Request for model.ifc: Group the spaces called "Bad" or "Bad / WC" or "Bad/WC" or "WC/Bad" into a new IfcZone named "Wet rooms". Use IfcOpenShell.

First a look at what the model holds.

```python
import ifcopenshell

model = ifcopenshell.open("model.ifc")
print(model.schema)
seen = {}
for space in model.by_type("IfcSpace"):
    seen[space.LongName] = seen.get(space.LongName, 0) + 1
for name, count in sorted(seen.items(), key=str):
    print(count, "x", name)
print("zones:", [z.Name for z in model.by_type("IfcZone")][:20])
```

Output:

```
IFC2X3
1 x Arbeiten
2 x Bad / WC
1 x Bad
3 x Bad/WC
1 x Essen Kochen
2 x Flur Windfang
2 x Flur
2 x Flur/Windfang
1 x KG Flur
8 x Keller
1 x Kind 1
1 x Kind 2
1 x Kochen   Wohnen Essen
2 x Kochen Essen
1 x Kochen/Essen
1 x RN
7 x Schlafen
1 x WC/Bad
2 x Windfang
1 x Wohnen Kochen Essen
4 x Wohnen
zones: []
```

```python
import ifcopenshell
import ifcopenshell.api.group
import ifcopenshell.api.root

model = ifcopenshell.open("model.ifc")

names = {"Bad", "Bad / WC", "Bad/WC", "WC/Bad"}
spaces = [s for s in model.by_type("IfcSpace") if s.LongName in names]

zone = ifcopenshell.api.root.create_entity(model, ifc_class="IfcZone", name="Wet rooms")
ifcopenshell.api.group.assign_group(model, products=spaces, group=zone)
print(len(spaces), "spaces in", zone.Name)

model.write("model_v2.ifc")
```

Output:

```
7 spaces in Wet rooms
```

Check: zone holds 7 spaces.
